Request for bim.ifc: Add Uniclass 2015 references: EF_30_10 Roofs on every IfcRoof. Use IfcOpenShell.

First a look at what the model holds.

```python
import ifcopenshell

model = ifcopenshell.open("bim.ifc")
print(model.schema)
print("classifications:", [c.Name for c in model.by_type("IfcClassification")])
for ifc_class in ("IfcDoor", "IfcRoof", "IfcStair", "IfcWall", "IfcWindow"):
    print(ifc_class, len(model.by_type(ifc_class)))
```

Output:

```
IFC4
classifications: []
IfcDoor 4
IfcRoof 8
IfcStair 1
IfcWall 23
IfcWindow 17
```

```python
import ifcopenshell
import ifcopenshell.api.classification

model = ifcopenshell.open("bim.ifc")

system = ifcopenshell.api.classification.add_classification(model, classification="Uniclass 2015")

codes = {
    "IfcRoof": ("EF_30_10", "Roofs"),
}
for ifc_class, (code, name) in codes.items():
    products = model.by_type(ifc_class)
    ifcopenshell.api.classification.add_reference(
        model, products=products, classification=system, identification=code, name=name
    )
    print(code, len(products))

model.write("bim_rev.ifc")
```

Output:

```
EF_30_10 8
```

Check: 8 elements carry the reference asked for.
